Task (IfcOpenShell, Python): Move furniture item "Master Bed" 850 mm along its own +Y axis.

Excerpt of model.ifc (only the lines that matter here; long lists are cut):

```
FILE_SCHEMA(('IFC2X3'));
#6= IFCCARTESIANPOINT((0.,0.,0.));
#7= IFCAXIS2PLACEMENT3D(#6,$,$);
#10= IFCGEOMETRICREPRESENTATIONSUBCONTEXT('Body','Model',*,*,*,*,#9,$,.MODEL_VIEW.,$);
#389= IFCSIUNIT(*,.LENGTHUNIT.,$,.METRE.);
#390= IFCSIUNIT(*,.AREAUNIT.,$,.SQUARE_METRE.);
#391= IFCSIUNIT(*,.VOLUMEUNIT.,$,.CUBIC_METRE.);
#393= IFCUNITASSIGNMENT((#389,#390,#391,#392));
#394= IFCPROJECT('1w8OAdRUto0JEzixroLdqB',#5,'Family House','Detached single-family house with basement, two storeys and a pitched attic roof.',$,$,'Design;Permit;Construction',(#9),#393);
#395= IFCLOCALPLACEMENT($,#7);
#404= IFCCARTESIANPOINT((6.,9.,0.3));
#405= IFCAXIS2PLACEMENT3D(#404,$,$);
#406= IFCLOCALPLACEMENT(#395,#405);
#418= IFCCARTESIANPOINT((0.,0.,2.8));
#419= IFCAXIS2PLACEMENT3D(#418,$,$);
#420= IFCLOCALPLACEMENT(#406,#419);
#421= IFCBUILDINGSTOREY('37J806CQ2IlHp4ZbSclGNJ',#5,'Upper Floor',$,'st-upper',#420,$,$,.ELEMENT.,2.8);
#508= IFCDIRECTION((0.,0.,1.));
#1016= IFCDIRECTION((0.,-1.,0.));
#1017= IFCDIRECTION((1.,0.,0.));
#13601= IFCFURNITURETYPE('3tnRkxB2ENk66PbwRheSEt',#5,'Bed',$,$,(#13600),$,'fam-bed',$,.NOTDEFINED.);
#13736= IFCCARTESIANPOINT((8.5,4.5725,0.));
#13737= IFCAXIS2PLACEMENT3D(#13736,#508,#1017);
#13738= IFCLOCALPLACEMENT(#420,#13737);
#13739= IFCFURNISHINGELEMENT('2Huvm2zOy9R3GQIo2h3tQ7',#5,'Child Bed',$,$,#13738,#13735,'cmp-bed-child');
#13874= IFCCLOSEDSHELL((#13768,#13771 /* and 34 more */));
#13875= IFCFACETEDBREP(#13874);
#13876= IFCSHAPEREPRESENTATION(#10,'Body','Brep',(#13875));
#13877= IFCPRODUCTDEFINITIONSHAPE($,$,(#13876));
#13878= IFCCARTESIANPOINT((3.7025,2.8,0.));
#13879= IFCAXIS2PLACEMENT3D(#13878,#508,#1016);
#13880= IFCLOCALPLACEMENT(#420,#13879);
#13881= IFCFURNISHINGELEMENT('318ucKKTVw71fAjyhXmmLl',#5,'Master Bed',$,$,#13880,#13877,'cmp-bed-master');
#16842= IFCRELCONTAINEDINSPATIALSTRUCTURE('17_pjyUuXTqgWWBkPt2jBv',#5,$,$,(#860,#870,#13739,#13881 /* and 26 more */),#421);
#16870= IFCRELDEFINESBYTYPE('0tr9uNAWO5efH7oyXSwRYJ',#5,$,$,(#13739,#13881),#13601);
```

```python
import ifcopenshell
import ifcopenshell.api.geometry
import ifcopenshell.util.placement

model = ifcopenshell.open("model.ifc")

item = model.by_guid("318ucKKTVw71fAjyhXmmLl")
matrix = ifcopenshell.util.placement.get_local_placement(item.ObjectPlacement)
matrix[:3, 3] += matrix[:3, 1] * 0.85
ifcopenshell.api.geometry.edit_object_placement(model, product=item, matrix=matrix, is_si=False)

print(ifcopenshell.util.placement.get_local_placement(item.ObjectPlacement).round(3) + 0.0)

model.write("model-out.ifc")
```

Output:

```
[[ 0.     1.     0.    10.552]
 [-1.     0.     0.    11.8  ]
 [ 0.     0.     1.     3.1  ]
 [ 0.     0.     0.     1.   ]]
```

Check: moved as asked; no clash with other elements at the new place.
